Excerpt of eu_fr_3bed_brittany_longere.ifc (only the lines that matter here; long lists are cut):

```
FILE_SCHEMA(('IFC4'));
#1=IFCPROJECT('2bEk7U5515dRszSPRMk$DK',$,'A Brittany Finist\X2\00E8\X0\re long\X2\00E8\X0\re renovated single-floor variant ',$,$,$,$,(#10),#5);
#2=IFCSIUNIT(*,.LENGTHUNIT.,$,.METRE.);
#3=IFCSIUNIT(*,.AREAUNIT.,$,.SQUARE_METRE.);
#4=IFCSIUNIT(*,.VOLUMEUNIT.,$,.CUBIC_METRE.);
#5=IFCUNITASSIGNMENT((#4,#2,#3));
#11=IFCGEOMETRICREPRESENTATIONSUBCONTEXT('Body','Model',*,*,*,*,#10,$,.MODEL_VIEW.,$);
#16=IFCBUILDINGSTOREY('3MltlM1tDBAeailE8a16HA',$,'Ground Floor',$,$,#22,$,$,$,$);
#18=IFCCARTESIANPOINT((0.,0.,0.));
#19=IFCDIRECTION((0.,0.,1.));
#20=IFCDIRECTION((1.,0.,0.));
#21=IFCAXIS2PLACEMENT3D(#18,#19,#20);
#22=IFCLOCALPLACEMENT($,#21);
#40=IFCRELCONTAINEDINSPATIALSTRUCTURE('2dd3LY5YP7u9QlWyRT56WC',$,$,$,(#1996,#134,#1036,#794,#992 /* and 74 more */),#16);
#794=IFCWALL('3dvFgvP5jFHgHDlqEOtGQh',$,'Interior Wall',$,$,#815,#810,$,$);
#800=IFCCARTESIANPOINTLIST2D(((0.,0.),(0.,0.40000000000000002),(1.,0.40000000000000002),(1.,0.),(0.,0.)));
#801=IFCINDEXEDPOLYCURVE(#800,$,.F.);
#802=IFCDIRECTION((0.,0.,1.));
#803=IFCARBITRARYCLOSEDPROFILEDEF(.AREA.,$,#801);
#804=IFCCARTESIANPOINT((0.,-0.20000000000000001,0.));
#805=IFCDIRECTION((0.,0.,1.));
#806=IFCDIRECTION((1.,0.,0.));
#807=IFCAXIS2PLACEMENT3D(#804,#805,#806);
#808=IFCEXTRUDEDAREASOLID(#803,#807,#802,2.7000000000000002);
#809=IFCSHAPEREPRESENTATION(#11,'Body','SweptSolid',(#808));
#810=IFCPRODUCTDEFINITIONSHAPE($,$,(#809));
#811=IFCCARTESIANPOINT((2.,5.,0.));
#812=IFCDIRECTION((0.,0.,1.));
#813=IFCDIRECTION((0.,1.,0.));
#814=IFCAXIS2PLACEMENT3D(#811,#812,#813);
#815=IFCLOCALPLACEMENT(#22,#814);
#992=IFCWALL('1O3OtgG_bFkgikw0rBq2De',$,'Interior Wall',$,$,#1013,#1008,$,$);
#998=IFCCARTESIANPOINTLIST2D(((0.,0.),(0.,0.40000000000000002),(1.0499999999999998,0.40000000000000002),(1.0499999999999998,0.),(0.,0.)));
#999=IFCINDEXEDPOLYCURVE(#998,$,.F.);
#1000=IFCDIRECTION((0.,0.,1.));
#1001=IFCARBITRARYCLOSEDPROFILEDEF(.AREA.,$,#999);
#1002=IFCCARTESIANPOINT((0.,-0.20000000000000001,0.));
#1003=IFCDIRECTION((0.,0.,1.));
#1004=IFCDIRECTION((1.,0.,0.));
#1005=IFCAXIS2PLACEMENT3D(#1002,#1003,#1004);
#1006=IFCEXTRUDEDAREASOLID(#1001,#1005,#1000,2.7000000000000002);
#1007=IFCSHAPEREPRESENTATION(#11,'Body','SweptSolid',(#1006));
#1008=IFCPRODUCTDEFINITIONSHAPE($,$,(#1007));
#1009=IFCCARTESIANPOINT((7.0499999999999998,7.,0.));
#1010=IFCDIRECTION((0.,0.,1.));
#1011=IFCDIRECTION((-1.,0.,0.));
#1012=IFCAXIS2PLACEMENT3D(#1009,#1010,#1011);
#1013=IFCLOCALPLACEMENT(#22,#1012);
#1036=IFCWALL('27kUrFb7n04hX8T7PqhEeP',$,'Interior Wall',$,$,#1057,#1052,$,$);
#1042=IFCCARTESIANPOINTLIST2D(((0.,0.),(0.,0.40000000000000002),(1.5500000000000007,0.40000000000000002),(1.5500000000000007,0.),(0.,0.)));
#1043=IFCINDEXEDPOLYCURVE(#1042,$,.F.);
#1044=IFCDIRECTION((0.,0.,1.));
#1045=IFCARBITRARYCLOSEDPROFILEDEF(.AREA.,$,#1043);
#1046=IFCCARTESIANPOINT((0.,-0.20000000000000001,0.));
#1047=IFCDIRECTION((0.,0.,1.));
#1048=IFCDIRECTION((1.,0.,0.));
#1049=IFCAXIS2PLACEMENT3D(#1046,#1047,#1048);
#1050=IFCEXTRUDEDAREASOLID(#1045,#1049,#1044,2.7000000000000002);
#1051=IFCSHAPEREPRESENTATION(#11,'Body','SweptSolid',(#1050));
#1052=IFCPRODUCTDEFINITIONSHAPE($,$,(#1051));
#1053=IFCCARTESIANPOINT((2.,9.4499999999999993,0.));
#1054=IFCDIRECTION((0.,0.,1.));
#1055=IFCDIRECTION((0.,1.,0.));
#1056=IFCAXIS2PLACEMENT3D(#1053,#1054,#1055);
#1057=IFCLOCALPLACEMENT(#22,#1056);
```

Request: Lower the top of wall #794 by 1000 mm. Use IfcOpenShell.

```python
import ifcopenshell
import ifcopenshell.geom
import ifcopenshell.util.representation
import ifcopenshell.util.shape
import ifcopenshell.util.unit

model = ifcopenshell.open("eu_fr_3bed_brittany_longere.ifc")
unit_scale = ifcopenshell.util.unit.calculate_unit_scale(model)
settings = ifcopenshell.geom.settings()


def volume(element):
    """Net volume in cubic metres, openings subtracted."""
    shape = ifcopenshell.geom.create_shape(settings, element)
    return ifcopenshell.util.shape.get_volume(shape.geometry)


wall = model.by_guid("3dvFgvP5jFHgHDlqEOtGQh")
before = volume(wall)

body = ifcopenshell.util.representation.get_representation(wall, "Model", "Body")
solid = body.Items[0]
old_height = solid.Depth
solid.Depth -= 1 / unit_scale
after = volume(wall)

print(f"height {old_height:g} -> {solid.Depth:g}, volume {before:.3f} -> {after:.3f} m3")

model.write("eu_fr_3bed_brittany_longere_edited.ifc")
```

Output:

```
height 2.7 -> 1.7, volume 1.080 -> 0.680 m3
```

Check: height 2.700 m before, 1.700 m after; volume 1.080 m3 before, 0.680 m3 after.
